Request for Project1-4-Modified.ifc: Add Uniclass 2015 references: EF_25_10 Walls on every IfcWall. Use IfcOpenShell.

First a look at what the model holds.

```python
import ifcopenshell

model = ifcopenshell.open("Project1-4-Modified.ifc")
print(model.schema)
print("classifications:", [c.Name for c in model.by_type("IfcClassification")])
for ifc_class in ("IfcDoor", "IfcRoof", "IfcStair", "IfcWall", "IfcWindow"):
    print(ifc_class, len(model.by_type(ifc_class)))
```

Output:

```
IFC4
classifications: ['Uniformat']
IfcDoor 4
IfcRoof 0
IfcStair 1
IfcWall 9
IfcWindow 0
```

```python
import ifcopenshell
import ifcopenshell.api.classification

model = ifcopenshell.open("Project1-4-Modified.ifc")

system = ifcopenshell.api.classification.add_classification(model, classification="Uniclass 2015")

codes = {
    "IfcWall": ("EF_25_10", "Walls"),
}
for ifc_class, (code, name) in codes.items():
    products = model.by_type(ifc_class)
    ifcopenshell.api.classification.add_reference(
        model, products=products, classification=system, identification=code, name=name
    )
    print(code, len(products))

model.write("Project1-4-Modified_edited.ifc")
```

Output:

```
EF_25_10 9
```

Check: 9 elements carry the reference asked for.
